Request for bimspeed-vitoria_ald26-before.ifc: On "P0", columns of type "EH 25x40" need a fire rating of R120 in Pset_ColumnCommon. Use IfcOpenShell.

First a look at what the model holds.

```python
import ifcopenshell
import ifcopenshell.util.element

model = ifcopenshell.open("bimspeed-vitoria_ald26-before.ifc")
print(model.schema)
storey = next(s for s in model.by_type("IfcBuildingStorey") if s.Name == "P0")
columns = [e for e in ifcopenshell.util.element.get_decomposition(storey) if e.is_a("IfcColumn")]
seen = {}
for e in columns:
    element_type = ifcopenshell.util.element.get_type(e)
    key = (element_type.Name if element_type != e and element_type else None, ifcopenshell.util.element.get_pset(e, "Pset_ColumnCommon", "FireRating"))
    seen[key] = seen.get(key, 0) + 1
for (name, value), count in sorted(seen.items(), key=str):
    print(count, "x", name, "|", value)
```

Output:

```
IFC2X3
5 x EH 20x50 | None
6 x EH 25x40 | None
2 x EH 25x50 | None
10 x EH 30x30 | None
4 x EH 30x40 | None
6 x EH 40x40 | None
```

```python
import ifcopenshell
import ifcopenshell.api.pset
import ifcopenshell.util.element

model = ifcopenshell.open("bimspeed-vitoria_ald26-before.ifc")

storey = next(s for s in model.by_type("IfcBuildingStorey") if s.Name == "P0")
columns = [e for e in ifcopenshell.util.element.get_decomposition(storey) if e.is_a("IfcColumn")]

count = 0
for e in columns:
    element_type = ifcopenshell.util.element.get_type(e)
    if element_type in (None, e) or element_type.Name != "EH 25x40":
        continue
    # add_pset returns the element's existing set when there is one.
    pset = ifcopenshell.api.pset.add_pset(model, product=e, name="Pset_ColumnCommon")
    ifcopenshell.api.pset.edit_pset(model, pset=pset, properties={"FireRating": "R120"})
    count += 1

print(count, "columns updated")

model.write("bimspeed-vitoria_ald26-before_rev.ifc")
```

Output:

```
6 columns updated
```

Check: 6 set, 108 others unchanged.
